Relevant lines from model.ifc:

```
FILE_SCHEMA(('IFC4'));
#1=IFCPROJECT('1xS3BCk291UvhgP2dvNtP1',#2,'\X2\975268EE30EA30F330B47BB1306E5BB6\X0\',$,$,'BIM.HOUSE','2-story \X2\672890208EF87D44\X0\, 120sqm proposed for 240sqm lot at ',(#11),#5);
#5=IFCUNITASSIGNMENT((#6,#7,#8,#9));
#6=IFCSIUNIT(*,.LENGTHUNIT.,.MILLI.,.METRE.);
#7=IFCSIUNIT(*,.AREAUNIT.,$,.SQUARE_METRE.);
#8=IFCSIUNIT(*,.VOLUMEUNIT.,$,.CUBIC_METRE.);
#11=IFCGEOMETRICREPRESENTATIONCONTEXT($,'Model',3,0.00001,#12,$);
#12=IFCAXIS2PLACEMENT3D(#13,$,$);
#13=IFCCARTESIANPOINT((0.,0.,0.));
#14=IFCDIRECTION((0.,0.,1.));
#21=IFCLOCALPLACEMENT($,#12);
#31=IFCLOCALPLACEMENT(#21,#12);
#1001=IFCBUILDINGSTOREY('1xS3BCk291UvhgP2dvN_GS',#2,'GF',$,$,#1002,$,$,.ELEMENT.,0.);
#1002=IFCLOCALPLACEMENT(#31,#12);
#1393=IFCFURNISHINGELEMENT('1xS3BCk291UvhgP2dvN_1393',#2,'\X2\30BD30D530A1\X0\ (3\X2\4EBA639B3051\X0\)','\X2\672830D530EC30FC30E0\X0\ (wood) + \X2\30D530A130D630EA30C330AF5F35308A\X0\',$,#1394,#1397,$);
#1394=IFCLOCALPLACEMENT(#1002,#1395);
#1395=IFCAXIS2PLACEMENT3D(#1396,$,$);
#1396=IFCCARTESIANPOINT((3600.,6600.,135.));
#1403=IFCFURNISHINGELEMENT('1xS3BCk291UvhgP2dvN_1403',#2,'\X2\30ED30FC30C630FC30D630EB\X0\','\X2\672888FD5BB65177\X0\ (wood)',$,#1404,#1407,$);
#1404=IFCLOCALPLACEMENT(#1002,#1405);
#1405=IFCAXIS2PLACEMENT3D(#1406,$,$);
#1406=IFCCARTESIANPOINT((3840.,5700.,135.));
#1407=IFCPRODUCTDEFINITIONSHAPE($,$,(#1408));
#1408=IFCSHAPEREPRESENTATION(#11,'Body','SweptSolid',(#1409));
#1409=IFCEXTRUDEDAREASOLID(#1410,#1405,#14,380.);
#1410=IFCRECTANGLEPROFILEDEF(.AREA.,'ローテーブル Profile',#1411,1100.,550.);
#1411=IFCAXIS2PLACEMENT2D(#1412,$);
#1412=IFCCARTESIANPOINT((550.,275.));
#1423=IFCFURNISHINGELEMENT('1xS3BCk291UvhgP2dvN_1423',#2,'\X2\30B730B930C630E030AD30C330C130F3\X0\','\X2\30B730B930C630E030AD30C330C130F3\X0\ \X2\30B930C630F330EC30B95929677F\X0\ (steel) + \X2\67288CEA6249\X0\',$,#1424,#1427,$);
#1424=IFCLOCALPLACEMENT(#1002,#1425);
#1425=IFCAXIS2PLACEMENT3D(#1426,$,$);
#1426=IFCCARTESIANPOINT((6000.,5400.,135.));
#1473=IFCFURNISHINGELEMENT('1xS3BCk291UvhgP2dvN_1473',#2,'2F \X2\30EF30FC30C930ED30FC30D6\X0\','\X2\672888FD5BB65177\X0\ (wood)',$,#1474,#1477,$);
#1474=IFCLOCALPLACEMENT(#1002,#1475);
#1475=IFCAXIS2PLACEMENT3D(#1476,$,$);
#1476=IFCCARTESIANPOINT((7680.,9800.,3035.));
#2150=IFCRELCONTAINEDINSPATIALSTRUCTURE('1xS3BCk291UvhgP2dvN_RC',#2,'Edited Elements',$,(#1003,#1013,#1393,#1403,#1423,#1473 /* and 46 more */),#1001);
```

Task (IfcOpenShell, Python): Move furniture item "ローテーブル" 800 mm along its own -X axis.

```python
import ifcopenshell
import ifcopenshell.api.geometry
import ifcopenshell.util.placement
import ifcopenshell.util.unit

model = ifcopenshell.open("model.ifc")
unit_scale = ifcopenshell.util.unit.calculate_unit_scale(model)

item = model.by_id(1403)
matrix = ifcopenshell.util.placement.get_local_placement(item.ObjectPlacement)
matrix[:3, 3] -= matrix[:3, 0] * 0.8 / unit_scale
ifcopenshell.api.geometry.edit_object_placement(model, product=item, matrix=matrix, is_si=False)

print(ifcopenshell.util.placement.get_local_placement(item.ObjectPlacement).round(3) + 0.0)

model.write("model_updated.ifc")
```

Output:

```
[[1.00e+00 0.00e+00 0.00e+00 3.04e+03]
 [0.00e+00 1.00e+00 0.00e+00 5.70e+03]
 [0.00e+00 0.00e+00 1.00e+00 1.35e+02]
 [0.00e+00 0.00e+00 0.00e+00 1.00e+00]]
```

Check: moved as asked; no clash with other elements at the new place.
